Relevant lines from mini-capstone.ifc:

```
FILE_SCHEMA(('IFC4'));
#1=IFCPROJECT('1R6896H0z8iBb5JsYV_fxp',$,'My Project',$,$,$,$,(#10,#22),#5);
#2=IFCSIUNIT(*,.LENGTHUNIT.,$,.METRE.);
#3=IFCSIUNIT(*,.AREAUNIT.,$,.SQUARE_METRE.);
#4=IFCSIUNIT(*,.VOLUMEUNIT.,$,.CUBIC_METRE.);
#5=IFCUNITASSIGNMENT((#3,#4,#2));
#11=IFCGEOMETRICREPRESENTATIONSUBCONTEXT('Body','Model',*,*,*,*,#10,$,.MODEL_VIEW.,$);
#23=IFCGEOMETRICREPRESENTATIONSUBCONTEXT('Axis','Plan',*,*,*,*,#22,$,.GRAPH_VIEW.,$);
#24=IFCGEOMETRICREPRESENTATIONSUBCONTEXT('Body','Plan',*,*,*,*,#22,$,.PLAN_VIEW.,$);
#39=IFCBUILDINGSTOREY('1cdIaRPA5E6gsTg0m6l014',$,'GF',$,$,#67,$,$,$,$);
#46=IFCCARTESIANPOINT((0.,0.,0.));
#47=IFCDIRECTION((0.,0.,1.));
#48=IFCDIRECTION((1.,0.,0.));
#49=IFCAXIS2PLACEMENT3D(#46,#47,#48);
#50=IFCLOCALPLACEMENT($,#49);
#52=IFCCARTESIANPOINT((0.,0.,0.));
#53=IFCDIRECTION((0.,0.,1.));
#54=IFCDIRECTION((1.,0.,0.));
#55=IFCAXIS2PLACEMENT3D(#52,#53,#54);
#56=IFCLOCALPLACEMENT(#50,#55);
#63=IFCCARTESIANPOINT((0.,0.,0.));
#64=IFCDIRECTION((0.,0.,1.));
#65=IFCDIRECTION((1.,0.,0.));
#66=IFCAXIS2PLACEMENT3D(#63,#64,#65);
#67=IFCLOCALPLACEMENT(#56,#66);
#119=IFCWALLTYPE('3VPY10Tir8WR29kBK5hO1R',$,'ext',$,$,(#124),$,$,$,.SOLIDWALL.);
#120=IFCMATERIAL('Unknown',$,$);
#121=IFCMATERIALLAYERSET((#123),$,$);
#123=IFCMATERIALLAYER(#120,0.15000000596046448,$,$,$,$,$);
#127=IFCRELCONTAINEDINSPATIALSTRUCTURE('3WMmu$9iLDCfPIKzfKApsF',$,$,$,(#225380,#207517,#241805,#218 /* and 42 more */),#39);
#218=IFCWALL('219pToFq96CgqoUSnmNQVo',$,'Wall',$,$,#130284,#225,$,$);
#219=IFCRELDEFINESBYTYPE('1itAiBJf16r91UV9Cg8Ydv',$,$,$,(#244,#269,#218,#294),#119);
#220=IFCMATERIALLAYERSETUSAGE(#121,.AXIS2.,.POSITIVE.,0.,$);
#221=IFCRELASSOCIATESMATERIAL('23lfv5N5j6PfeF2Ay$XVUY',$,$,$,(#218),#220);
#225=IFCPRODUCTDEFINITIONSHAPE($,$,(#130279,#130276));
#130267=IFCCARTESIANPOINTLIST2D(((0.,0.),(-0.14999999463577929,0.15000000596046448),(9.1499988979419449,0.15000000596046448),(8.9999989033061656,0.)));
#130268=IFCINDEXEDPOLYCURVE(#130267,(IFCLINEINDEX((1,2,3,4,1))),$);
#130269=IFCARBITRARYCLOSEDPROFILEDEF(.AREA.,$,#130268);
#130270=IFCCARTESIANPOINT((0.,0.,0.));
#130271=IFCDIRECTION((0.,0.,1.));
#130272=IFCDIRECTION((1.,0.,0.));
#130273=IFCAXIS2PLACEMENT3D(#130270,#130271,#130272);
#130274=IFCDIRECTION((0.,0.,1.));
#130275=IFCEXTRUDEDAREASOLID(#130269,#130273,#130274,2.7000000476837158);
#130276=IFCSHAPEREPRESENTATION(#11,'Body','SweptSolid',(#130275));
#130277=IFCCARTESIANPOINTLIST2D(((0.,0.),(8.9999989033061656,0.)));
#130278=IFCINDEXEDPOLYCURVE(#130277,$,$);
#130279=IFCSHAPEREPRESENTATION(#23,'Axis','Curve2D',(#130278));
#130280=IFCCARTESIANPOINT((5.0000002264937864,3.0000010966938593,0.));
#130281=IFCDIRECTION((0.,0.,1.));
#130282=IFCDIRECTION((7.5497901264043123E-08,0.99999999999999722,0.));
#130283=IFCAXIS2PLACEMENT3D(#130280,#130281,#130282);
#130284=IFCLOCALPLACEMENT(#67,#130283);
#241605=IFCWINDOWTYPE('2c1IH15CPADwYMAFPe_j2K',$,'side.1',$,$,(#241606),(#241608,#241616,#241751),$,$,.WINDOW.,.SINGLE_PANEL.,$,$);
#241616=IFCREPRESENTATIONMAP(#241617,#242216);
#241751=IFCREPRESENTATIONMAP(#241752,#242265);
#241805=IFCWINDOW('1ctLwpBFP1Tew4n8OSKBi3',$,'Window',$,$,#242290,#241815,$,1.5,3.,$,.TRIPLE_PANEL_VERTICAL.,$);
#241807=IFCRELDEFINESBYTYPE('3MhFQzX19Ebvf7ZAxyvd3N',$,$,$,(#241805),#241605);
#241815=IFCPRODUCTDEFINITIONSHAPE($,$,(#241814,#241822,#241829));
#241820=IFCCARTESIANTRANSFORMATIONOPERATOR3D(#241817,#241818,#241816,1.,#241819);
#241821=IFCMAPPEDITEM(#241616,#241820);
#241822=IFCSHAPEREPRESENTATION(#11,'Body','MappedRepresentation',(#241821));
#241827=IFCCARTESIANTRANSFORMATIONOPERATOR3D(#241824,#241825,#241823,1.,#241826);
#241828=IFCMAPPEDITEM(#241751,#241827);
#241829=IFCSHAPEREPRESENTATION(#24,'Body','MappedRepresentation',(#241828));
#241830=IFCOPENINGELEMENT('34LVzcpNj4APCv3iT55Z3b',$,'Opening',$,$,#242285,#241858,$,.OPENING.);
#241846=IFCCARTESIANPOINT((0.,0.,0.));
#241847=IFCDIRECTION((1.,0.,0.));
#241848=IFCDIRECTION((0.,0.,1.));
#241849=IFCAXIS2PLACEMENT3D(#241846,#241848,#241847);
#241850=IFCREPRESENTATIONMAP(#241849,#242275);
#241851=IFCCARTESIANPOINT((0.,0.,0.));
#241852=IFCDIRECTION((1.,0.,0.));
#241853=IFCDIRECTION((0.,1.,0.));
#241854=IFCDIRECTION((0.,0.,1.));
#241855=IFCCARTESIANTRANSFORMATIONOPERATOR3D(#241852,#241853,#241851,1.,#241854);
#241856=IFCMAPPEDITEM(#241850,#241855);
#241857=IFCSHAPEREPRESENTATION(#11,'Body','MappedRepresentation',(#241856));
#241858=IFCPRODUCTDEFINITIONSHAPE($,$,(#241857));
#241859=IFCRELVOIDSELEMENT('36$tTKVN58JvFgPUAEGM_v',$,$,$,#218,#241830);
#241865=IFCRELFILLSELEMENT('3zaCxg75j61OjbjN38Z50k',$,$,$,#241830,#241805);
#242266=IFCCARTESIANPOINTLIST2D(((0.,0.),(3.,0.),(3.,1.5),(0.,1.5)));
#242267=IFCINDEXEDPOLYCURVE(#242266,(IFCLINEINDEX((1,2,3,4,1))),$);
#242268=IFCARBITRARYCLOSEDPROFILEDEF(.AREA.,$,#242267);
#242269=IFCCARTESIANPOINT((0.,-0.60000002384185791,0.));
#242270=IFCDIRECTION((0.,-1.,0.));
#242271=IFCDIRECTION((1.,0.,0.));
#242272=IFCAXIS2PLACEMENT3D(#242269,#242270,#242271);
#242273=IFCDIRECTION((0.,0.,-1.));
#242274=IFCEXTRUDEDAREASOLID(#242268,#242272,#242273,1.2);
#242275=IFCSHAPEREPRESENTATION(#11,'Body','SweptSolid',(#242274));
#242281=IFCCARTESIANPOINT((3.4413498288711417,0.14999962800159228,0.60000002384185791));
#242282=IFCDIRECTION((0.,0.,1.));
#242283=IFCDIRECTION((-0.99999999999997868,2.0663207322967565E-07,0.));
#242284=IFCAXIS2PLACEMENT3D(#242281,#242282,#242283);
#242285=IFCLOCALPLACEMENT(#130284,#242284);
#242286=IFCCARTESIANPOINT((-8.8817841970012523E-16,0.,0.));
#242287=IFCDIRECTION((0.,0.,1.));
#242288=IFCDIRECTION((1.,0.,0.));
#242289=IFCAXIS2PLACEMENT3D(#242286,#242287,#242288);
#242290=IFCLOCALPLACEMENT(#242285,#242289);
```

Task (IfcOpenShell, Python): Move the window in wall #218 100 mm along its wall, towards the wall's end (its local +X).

```python
import ifcopenshell
import ifcopenshell.api.geometry
import ifcopenshell.util.placement
import ifcopenshell.util.unit

model = ifcopenshell.open("mini-capstone.ifc")
unit_scale = ifcopenshell.util.unit.calculate_unit_scale(model)

window = model.by_id(241805)
opening = window.FillsVoids[0].RelatingOpeningElement
wall = opening.VoidsElements[0].RelatingBuildingElement

wall_matrix = ifcopenshell.util.placement.get_local_placement(wall.ObjectPlacement)
shift = wall_matrix[:3, 0] * 0.1 / unit_scale
before = ifcopenshell.util.placement.get_local_placement(window.ObjectPlacement)[:3, 3].copy()

# The window is placed relative to its opening, so it follows when the opening moves.
matrix = ifcopenshell.util.placement.get_local_placement(opening.ObjectPlacement)
matrix[:3, 3] += shift
ifcopenshell.api.geometry.edit_object_placement(
    model, product=opening, matrix=matrix, is_si=False, should_transform_children=True
)

after = ifcopenshell.util.placement.get_local_placement(window.ObjectPlacement)[:3, 3]
print("window moved by", (after - before).round(3) + 0.0)

model.write("mini-capstone_rev.ifc")
```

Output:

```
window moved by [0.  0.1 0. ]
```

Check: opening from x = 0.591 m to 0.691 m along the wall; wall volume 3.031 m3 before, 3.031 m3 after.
